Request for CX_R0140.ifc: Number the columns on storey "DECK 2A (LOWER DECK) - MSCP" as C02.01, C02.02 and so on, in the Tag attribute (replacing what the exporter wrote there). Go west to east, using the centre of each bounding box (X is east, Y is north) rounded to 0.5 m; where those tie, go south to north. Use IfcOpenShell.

First a look at what the model holds.

```python
import ifcopenshell
import ifcopenshell.util.element
import ifcopenshell.util.placement

model = ifcopenshell.open("CX_R0140.ifc")
print(model.schema)
storey = next(s for s in model.by_type("IfcBuildingStorey") if s.Name == "DECK 2A (LOWER DECK) - MSCP")
columns = [e for e in ifcopenshell.util.element.get_decomposition(storey) if e.is_a("IfcColumn")]
for e in sorted(columns, key=lambda e: e.id()):
    origin = ifcopenshell.util.placement.get_local_placement(e.ObjectPlacement)[:3, 3]
    print(e.id(), e.Tag, e.Name, origin.round(2) + 0.0, sep=" | ")
```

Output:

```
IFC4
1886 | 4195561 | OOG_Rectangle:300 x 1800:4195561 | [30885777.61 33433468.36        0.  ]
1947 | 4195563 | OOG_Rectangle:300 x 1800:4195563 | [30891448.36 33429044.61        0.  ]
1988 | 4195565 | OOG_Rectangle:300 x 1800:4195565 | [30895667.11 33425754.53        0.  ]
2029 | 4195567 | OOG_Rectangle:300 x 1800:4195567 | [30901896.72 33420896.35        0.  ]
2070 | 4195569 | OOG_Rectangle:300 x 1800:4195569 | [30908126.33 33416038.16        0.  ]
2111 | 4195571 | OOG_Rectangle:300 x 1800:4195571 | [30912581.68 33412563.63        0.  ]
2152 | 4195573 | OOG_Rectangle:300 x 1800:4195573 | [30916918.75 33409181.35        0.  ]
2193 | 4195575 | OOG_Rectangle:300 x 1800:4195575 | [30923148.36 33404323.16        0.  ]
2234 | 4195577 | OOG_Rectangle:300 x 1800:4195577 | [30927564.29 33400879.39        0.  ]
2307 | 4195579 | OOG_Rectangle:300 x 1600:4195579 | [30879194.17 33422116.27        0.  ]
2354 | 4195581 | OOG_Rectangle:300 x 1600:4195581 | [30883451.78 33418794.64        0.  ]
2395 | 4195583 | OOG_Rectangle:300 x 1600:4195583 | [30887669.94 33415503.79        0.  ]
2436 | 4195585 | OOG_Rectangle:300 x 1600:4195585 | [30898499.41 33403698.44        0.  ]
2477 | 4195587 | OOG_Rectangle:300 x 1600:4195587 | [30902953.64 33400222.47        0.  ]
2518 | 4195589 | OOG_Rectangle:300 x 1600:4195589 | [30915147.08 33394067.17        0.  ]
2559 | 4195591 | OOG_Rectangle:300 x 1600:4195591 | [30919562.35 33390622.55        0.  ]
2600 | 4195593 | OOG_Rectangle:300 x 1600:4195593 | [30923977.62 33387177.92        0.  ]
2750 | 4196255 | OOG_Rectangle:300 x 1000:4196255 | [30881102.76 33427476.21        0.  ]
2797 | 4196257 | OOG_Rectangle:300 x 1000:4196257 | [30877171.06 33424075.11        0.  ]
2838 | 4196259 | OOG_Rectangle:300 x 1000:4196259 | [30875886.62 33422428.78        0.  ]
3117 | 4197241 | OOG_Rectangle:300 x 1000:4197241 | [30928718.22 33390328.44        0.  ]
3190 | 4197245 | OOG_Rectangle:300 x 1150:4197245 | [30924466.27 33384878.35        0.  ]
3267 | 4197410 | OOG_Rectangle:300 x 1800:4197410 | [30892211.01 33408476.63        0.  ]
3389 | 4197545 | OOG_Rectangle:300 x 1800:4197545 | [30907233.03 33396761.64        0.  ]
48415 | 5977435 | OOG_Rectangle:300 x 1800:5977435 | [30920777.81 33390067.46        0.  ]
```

```python
import ifcopenshell
import ifcopenshell.geom
import ifcopenshell.util.element
import ifcopenshell.util.shape

model = ifcopenshell.open("CX_R0140.ifc")
settings = ifcopenshell.geom.settings()
settings.set("use-world-coords", True)


def centre(element):
    shape = ifcopenshell.geom.create_shape(settings, element)
    return ifcopenshell.util.shape.get_bbox_centroid(shape.geometry)


storey = next(s for s in model.by_type("IfcBuildingStorey") if s.Name == "DECK 2A (LOWER DECK) - MSCP")
columns = [e for e in ifcopenshell.util.element.get_decomposition(storey) if e.is_a("IfcColumn")]

# Insertion points can sit at a corner or the storey origin, so sort by the geometry (in metres).
centres = {e: centre(e) for e in columns}
columns.sort(key=lambda e: (round(centres[e][0] / 0.5), centres[e][1]))

for i, e in enumerate(columns, start=1):
    number = f"C02.{i:02d}"
    e.Tag = number
    print(e.id(), number)

model.write("CX_R0140_rev.ifc")
```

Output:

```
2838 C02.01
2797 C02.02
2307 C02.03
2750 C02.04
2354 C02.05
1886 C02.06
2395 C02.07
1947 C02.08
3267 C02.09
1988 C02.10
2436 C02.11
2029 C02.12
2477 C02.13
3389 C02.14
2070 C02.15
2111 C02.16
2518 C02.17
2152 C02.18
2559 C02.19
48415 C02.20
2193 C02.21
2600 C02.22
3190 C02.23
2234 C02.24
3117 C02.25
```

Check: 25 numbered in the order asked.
